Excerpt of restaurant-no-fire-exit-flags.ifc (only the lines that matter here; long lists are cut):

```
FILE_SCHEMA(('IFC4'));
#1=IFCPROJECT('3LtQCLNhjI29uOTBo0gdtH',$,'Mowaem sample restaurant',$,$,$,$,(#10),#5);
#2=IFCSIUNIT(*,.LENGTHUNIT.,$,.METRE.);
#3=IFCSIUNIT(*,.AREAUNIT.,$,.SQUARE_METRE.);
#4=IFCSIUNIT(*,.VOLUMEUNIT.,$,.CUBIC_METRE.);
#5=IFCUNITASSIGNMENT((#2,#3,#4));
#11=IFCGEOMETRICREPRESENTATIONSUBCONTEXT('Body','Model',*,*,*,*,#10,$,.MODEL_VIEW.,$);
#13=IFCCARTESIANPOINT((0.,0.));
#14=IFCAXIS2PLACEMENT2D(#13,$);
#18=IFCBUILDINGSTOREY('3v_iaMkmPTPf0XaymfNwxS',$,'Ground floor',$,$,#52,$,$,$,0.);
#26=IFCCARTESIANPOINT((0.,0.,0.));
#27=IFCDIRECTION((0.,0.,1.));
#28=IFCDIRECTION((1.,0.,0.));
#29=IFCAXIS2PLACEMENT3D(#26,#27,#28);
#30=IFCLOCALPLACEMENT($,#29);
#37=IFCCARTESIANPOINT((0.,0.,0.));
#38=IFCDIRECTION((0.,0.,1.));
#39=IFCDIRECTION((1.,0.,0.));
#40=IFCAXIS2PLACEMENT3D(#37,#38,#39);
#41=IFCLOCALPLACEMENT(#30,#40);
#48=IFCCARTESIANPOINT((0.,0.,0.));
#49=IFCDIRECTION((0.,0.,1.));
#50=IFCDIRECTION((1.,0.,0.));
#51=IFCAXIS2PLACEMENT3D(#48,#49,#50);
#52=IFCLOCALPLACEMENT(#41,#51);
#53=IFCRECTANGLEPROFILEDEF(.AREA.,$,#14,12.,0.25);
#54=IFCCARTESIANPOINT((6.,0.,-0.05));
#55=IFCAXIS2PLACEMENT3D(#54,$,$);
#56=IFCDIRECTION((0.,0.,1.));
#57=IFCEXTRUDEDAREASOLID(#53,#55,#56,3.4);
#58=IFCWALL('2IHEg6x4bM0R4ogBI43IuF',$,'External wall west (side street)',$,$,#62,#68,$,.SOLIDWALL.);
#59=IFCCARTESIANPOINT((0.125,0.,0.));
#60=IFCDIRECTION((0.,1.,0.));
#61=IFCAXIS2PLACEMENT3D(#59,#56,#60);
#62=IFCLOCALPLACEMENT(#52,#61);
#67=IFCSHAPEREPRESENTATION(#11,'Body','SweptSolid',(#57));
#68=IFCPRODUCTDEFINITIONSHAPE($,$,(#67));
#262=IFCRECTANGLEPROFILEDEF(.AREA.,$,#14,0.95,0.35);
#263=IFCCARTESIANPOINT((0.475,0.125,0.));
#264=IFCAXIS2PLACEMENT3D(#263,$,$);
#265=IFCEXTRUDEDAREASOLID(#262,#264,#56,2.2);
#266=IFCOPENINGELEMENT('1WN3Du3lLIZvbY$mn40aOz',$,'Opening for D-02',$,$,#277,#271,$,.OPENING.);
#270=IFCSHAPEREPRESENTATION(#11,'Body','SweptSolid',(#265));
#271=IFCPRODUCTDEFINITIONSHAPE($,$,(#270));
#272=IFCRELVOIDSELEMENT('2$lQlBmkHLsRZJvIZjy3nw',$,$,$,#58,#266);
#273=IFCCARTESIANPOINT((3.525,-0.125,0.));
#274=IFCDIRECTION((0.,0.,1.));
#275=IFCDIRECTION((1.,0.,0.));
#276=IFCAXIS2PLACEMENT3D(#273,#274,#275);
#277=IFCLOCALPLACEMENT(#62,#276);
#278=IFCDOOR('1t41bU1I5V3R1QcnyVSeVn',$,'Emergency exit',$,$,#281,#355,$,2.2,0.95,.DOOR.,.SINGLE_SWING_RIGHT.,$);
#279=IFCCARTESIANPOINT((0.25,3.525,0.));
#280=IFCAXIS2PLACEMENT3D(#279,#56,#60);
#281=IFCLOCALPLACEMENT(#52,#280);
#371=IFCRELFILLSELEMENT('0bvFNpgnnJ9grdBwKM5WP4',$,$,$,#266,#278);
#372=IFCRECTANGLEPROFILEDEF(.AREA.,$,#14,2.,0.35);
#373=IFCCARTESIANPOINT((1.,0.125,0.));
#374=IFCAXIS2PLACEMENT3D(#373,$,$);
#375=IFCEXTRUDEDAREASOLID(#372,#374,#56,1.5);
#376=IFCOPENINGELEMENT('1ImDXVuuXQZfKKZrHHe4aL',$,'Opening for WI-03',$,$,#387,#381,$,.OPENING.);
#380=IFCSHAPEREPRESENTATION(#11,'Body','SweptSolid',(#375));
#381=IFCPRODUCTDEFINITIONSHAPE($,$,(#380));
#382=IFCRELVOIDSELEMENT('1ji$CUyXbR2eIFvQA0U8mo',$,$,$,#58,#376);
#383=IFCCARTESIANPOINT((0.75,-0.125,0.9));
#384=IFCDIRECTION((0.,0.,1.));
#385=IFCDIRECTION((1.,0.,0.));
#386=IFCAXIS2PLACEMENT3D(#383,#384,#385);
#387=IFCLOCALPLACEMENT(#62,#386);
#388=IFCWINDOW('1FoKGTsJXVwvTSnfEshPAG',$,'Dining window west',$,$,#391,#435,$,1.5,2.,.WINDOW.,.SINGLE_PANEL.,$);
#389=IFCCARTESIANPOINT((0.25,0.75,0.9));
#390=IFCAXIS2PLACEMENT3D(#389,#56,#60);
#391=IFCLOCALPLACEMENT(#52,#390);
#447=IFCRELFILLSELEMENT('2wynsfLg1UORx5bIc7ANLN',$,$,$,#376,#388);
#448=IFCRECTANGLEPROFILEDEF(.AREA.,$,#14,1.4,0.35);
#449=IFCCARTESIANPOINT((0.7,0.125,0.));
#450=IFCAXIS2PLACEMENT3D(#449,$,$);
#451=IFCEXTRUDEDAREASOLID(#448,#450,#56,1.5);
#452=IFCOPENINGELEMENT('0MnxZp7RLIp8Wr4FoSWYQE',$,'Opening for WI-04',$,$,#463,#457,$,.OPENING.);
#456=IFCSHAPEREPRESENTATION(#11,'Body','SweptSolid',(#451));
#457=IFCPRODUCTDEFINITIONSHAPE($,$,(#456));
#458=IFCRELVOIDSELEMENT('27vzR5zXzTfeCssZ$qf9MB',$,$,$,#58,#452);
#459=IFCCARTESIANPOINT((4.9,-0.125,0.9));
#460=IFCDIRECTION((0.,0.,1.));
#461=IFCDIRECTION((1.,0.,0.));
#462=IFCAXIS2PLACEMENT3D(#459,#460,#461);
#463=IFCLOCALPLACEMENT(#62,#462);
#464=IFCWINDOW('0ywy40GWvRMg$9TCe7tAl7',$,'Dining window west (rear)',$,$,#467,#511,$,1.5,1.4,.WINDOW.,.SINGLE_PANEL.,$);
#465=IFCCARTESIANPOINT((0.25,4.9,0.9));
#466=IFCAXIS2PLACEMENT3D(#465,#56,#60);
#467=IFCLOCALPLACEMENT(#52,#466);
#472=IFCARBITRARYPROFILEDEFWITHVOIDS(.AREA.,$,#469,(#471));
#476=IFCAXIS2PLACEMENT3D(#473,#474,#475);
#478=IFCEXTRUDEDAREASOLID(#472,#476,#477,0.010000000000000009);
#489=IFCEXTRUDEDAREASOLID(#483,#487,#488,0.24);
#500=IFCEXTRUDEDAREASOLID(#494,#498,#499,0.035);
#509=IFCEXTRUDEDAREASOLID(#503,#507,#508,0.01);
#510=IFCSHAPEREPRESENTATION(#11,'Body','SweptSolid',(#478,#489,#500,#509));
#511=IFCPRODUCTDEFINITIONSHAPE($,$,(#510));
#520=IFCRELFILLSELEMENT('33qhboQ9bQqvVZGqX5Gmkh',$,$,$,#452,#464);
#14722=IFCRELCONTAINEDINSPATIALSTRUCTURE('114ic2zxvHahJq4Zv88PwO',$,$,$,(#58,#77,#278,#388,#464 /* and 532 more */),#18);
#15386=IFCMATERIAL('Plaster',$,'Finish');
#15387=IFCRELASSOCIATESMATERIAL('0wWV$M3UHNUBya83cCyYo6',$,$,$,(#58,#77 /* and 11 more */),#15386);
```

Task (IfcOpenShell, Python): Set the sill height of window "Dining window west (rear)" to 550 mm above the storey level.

```python
import numpy as np
import ifcopenshell
import ifcopenshell.api.geometry
import ifcopenshell.geom
import ifcopenshell.util.element
import ifcopenshell.util.placement
import ifcopenshell.util.shape
import ifcopenshell.util.unit

model = ifcopenshell.open("restaurant-no-fire-exit-flags.ifc")
unit_scale = ifcopenshell.util.unit.calculate_unit_scale(model)

window = model.by_guid("0ywy40GWvRMg$9TCe7tAl7")
opening = window.FillsVoids[0].RelatingOpeningElement
storey = ifcopenshell.util.element.get_container(window, ifc_class="IfcBuildingStorey")
level = ifcopenshell.util.placement.get_local_placement(storey.ObjectPlacement)[2, 3]

# The opening's origin need not be at the sill, so measure its lowest point.
shape = ifcopenshell.geom.create_shape(ifcopenshell.geom.settings(), opening)
bottom = ifcopenshell.util.shape.get_shape_bottom_elevation(shape, shape.geometry) / unit_scale
dz = level + 0.55 / unit_scale - bottom

shift = np.array([0.0, 0.0, dz])
# The window is not placed relative to its opening, so move both.
for product in (opening, window):
    matrix = ifcopenshell.util.placement.get_local_placement(product.ObjectPlacement)
    matrix[:3, 3] += shift
    ifcopenshell.api.geometry.edit_object_placement(model, product=product, matrix=matrix, is_si=False)

print(f"moved by {dz * unit_scale:+.3f} m")

model.write("restaurant-no-fire-exit-flags_rev.ifc")
```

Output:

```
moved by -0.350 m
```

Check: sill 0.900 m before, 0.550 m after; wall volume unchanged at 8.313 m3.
